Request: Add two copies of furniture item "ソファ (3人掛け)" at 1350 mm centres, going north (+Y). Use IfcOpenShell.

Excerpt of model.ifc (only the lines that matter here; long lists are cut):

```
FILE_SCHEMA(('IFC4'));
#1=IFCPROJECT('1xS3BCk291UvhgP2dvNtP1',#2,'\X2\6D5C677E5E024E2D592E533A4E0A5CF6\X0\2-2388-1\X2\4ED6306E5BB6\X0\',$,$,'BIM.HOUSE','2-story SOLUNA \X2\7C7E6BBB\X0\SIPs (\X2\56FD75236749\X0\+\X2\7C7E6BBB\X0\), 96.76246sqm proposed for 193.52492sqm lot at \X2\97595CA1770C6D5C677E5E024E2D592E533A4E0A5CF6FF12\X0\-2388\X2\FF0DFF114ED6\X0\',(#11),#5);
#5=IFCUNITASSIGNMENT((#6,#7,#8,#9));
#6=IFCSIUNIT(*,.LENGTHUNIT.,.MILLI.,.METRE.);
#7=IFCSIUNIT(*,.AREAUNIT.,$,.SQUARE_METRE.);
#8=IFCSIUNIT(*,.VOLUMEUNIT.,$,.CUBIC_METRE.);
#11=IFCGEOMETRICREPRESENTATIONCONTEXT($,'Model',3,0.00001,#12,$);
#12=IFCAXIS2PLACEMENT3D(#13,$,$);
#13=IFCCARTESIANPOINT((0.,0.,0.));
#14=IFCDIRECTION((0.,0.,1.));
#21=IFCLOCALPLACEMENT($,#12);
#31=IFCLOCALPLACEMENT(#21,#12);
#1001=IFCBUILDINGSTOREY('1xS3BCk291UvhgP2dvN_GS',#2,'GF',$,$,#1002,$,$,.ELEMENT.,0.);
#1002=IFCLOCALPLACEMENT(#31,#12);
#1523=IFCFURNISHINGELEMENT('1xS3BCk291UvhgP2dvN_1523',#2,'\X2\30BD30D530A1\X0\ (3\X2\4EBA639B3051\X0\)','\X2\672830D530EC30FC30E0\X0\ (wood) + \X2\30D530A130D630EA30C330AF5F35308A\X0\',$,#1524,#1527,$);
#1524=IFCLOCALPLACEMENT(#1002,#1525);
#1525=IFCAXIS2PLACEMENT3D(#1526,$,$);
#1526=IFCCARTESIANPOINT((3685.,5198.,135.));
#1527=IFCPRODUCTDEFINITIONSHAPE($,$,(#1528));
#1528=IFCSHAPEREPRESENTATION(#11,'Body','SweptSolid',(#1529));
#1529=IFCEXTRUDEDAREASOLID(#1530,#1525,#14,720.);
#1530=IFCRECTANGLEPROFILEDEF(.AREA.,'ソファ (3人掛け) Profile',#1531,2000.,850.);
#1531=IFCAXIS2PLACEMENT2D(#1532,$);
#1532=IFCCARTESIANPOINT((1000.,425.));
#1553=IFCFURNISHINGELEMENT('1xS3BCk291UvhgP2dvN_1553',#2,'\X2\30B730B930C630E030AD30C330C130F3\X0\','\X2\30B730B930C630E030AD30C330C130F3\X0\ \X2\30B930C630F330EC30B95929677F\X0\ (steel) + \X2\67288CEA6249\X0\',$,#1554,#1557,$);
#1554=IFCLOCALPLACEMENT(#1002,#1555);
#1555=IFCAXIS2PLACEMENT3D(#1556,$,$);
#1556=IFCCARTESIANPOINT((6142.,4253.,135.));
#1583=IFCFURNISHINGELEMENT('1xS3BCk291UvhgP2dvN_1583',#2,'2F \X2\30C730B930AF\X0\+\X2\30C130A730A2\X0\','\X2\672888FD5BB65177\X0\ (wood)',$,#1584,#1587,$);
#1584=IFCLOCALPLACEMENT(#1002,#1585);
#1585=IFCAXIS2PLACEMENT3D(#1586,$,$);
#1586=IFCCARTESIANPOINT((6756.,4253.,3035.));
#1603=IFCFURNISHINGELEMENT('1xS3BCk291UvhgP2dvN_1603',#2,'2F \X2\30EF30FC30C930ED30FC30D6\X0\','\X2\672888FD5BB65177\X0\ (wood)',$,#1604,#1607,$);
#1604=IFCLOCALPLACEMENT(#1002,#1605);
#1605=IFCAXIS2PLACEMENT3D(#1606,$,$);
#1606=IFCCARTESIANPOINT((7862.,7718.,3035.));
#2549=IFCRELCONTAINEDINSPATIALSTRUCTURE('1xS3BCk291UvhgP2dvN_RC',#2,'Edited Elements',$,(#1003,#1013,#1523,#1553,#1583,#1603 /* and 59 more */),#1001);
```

```python
import numpy as np
import ifcopenshell
import ifcopenshell.api.geometry
import ifcopenshell.api.root
import ifcopenshell.util.element
import ifcopenshell.util.placement

model = ifcopenshell.open("model.ifc")


def reuse_history(source, copy):
    """copy_class also copies each property set's owner history, people and application; keep the originals."""
    for rel in copy.IsDefinedBy:
        if rel.is_a("IfcRelDefinesByProperties") and (history := rel.RelatingPropertyDefinition.OwnerHistory):
            rel.RelatingPropertyDefinition.OwnerHistory = source.OwnerHistory
            ifcopenshell.util.element.remove_deep2(model, history)


source = model.by_guid("1xS3BCk291UvhgP2dvN_1523")
base = ifcopenshell.util.placement.get_local_placement(source.ObjectPlacement)
step = np.array([0.0, 1.0, 0.0]) * 1350.0

for i in range(1, 3):
    copy = ifcopenshell.api.root.copy_class(model, product=source)
    copy.Representation = ifcopenshell.util.element.copy_deep(
        model, source.Representation, exclude=["IfcGeometricRepresentationContext", "IfcRepresentationMap"]
    )
    reuse_history(source, copy)
    matrix = base.copy()
    matrix[:3, 3] += i * step
    print("added at", matrix[:3, 3].round(3) + 0.0)
    ifcopenshell.api.geometry.edit_object_placement(model, product=copy, matrix=matrix, is_si=False)

model.write("model_v2.ifc")
```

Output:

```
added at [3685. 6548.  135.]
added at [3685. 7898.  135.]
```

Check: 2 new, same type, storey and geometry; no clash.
